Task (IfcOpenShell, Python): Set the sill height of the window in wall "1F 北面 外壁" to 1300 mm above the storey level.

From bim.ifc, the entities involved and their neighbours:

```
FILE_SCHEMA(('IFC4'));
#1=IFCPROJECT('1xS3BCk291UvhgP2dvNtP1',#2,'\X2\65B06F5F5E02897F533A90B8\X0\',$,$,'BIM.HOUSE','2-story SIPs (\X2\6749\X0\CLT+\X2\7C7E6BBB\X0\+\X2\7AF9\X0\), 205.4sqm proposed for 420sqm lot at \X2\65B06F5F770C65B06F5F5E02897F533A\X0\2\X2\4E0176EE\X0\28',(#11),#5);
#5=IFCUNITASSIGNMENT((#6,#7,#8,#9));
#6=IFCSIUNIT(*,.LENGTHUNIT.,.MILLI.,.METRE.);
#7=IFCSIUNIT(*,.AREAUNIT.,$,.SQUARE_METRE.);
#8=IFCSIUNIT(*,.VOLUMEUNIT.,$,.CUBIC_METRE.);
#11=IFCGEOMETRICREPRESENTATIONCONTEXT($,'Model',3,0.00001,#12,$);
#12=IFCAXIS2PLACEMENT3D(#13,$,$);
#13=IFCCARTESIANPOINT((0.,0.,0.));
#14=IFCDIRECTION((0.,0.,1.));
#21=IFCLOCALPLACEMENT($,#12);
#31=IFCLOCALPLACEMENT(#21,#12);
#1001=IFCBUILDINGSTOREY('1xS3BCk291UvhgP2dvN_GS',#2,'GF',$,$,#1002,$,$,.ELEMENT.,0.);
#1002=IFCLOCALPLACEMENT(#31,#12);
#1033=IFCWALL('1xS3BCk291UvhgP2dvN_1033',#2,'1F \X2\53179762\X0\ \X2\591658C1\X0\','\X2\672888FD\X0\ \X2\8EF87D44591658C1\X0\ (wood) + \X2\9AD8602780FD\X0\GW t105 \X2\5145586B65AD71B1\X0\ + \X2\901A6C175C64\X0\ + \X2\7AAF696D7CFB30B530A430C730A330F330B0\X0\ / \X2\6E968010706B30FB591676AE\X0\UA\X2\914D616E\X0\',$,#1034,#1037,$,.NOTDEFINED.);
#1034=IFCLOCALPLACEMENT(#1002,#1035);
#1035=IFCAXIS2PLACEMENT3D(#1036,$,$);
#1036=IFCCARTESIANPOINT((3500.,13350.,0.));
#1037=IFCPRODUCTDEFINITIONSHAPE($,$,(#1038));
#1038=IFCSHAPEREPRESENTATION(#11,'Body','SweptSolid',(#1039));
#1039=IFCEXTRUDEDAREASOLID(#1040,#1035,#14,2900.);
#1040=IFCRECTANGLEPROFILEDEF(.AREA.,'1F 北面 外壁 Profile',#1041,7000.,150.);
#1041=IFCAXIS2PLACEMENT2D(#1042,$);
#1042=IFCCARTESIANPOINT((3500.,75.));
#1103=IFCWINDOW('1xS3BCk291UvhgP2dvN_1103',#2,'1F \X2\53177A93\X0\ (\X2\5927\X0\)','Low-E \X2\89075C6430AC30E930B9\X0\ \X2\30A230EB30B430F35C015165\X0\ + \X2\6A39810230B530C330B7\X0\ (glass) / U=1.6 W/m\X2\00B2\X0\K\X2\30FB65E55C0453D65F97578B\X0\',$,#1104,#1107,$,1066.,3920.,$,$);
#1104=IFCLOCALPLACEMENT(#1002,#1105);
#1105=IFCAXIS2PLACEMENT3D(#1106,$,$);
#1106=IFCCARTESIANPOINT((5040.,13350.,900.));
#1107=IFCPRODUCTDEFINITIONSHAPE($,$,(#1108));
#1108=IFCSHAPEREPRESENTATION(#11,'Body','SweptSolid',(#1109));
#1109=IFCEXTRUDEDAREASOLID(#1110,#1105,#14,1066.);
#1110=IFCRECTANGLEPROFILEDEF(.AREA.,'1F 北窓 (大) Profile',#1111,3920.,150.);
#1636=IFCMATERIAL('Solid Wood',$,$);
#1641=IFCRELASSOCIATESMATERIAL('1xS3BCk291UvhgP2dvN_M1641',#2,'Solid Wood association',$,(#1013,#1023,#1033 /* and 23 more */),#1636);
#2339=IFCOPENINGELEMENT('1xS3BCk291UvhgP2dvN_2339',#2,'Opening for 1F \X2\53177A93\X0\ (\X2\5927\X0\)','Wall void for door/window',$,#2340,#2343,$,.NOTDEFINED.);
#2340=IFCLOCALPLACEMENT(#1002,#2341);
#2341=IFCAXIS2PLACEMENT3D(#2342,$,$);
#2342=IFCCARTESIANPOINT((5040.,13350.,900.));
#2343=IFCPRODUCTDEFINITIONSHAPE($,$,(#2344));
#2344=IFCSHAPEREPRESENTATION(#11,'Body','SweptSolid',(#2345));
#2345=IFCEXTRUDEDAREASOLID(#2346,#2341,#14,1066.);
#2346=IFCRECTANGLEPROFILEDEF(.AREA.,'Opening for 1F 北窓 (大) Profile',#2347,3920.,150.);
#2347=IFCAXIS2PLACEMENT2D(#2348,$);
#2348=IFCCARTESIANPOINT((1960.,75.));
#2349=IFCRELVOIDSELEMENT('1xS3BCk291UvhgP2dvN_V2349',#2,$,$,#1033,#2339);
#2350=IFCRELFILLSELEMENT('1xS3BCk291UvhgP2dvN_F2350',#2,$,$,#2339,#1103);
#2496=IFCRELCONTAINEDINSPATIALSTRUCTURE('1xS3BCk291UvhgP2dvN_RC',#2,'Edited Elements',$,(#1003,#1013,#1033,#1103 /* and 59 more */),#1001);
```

```python
import numpy as np
import ifcopenshell
import ifcopenshell.api.geometry
import ifcopenshell.geom
import ifcopenshell.util.element
import ifcopenshell.util.placement
import ifcopenshell.util.shape
import ifcopenshell.util.unit

model = ifcopenshell.open("bim.ifc")
unit_scale = ifcopenshell.util.unit.calculate_unit_scale(model)

window = model.by_guid("1xS3BCk291UvhgP2dvN_1103")
opening = window.FillsVoids[0].RelatingOpeningElement
storey = ifcopenshell.util.element.get_container(window, ifc_class="IfcBuildingStorey")
level = ifcopenshell.util.placement.get_local_placement(storey.ObjectPlacement)[2, 3]

# The opening's origin need not be at the sill, so measure its lowest point.
shape = ifcopenshell.geom.create_shape(ifcopenshell.geom.settings(), opening)
bottom = ifcopenshell.util.shape.get_shape_bottom_elevation(shape, shape.geometry) / unit_scale
dz = level + 1300.0 - bottom

shift = np.array([0.0, 0.0, dz])
# The window is not placed relative to its opening, so move both.
for product in (opening, window):
    matrix = ifcopenshell.util.placement.get_local_placement(product.ObjectPlacement)
    matrix[:3, 3] += shift
    ifcopenshell.api.geometry.edit_object_placement(model, product=product, matrix=matrix, is_si=False)

print(f"moved by {dz * unit_scale:+.3f} m")

model.write("bim_v2.ifc")
```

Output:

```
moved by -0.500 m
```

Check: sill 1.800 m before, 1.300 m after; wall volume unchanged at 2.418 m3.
